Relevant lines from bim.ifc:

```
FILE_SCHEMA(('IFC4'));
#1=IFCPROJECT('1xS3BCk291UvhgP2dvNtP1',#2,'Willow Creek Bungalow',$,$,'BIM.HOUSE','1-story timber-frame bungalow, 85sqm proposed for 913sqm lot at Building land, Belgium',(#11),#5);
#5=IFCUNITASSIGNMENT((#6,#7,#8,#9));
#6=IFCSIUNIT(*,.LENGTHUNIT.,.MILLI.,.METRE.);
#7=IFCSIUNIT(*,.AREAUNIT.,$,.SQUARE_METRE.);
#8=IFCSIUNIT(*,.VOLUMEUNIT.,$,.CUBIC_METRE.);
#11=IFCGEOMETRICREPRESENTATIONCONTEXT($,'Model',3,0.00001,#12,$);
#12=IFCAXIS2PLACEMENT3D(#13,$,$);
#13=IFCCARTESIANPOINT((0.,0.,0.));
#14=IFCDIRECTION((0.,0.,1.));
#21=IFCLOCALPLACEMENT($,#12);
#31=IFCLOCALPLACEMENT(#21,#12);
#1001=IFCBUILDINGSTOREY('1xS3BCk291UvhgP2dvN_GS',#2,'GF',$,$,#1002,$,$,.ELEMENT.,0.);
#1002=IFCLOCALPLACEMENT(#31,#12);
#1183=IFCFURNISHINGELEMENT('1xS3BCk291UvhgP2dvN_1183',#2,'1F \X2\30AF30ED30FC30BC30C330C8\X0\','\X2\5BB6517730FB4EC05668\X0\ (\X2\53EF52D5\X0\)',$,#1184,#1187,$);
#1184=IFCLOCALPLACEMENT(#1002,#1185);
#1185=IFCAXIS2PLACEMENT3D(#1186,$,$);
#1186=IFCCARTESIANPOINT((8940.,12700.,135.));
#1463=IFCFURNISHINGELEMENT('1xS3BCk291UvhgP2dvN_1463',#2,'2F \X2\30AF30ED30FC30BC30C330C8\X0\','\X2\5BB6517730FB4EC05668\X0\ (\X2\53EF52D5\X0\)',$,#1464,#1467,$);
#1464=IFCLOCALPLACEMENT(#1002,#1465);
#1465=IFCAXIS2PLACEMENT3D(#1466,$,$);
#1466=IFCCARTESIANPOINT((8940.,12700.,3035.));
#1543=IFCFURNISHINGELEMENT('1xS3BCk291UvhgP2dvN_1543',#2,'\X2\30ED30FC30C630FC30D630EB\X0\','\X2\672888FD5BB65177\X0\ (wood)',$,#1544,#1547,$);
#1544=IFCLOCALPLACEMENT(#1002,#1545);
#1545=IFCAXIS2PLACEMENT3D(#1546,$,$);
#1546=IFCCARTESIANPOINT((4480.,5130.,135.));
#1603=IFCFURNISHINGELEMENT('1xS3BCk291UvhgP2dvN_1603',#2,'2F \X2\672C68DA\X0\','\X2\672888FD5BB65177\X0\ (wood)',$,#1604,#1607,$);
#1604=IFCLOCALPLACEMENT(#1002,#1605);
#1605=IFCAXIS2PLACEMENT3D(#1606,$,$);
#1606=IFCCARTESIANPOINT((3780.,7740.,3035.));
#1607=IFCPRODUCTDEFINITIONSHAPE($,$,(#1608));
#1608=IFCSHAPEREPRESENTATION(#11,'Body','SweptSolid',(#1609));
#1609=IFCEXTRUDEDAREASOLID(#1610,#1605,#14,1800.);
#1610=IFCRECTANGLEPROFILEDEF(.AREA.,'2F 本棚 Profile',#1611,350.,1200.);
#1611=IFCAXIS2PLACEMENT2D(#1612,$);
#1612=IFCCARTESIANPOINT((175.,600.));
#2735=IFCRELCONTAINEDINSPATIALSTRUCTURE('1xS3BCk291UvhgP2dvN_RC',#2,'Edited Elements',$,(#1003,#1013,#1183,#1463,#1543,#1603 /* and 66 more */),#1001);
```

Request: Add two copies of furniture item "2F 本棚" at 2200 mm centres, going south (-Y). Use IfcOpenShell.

```python
import numpy as np
import ifcopenshell
import ifcopenshell.api.geometry
import ifcopenshell.api.root
import ifcopenshell.util.element
import ifcopenshell.util.placement

model = ifcopenshell.open("bim.ifc")


def reuse_history(source, copy):
    """copy_class also copies each property set's owner history, people and application; keep the originals."""
    for rel in copy.IsDefinedBy:
        if rel.is_a("IfcRelDefinesByProperties") and (history := rel.RelatingPropertyDefinition.OwnerHistory):
            rel.RelatingPropertyDefinition.OwnerHistory = source.OwnerHistory
            ifcopenshell.util.element.remove_deep2(model, history)


source = model.by_guid("1xS3BCk291UvhgP2dvN_1603")
base = ifcopenshell.util.placement.get_local_placement(source.ObjectPlacement)
step = np.array([0.0, -1.0, 0.0]) * 2200.0

for i in range(1, 3):
    copy = ifcopenshell.api.root.copy_class(model, product=source)
    copy.Representation = ifcopenshell.util.element.copy_deep(
        model, source.Representation, exclude=["IfcGeometricRepresentationContext", "IfcRepresentationMap"]
    )
    reuse_history(source, copy)
    matrix = base.copy()
    matrix[:3, 3] += i * step
    print("added at", matrix[:3, 3].round(3) + 0.0)
    ifcopenshell.api.geometry.edit_object_placement(model, product=copy, matrix=matrix, is_si=False)

model.write("bim_v2.ifc")
```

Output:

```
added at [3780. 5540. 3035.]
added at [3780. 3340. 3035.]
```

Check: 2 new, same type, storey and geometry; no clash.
